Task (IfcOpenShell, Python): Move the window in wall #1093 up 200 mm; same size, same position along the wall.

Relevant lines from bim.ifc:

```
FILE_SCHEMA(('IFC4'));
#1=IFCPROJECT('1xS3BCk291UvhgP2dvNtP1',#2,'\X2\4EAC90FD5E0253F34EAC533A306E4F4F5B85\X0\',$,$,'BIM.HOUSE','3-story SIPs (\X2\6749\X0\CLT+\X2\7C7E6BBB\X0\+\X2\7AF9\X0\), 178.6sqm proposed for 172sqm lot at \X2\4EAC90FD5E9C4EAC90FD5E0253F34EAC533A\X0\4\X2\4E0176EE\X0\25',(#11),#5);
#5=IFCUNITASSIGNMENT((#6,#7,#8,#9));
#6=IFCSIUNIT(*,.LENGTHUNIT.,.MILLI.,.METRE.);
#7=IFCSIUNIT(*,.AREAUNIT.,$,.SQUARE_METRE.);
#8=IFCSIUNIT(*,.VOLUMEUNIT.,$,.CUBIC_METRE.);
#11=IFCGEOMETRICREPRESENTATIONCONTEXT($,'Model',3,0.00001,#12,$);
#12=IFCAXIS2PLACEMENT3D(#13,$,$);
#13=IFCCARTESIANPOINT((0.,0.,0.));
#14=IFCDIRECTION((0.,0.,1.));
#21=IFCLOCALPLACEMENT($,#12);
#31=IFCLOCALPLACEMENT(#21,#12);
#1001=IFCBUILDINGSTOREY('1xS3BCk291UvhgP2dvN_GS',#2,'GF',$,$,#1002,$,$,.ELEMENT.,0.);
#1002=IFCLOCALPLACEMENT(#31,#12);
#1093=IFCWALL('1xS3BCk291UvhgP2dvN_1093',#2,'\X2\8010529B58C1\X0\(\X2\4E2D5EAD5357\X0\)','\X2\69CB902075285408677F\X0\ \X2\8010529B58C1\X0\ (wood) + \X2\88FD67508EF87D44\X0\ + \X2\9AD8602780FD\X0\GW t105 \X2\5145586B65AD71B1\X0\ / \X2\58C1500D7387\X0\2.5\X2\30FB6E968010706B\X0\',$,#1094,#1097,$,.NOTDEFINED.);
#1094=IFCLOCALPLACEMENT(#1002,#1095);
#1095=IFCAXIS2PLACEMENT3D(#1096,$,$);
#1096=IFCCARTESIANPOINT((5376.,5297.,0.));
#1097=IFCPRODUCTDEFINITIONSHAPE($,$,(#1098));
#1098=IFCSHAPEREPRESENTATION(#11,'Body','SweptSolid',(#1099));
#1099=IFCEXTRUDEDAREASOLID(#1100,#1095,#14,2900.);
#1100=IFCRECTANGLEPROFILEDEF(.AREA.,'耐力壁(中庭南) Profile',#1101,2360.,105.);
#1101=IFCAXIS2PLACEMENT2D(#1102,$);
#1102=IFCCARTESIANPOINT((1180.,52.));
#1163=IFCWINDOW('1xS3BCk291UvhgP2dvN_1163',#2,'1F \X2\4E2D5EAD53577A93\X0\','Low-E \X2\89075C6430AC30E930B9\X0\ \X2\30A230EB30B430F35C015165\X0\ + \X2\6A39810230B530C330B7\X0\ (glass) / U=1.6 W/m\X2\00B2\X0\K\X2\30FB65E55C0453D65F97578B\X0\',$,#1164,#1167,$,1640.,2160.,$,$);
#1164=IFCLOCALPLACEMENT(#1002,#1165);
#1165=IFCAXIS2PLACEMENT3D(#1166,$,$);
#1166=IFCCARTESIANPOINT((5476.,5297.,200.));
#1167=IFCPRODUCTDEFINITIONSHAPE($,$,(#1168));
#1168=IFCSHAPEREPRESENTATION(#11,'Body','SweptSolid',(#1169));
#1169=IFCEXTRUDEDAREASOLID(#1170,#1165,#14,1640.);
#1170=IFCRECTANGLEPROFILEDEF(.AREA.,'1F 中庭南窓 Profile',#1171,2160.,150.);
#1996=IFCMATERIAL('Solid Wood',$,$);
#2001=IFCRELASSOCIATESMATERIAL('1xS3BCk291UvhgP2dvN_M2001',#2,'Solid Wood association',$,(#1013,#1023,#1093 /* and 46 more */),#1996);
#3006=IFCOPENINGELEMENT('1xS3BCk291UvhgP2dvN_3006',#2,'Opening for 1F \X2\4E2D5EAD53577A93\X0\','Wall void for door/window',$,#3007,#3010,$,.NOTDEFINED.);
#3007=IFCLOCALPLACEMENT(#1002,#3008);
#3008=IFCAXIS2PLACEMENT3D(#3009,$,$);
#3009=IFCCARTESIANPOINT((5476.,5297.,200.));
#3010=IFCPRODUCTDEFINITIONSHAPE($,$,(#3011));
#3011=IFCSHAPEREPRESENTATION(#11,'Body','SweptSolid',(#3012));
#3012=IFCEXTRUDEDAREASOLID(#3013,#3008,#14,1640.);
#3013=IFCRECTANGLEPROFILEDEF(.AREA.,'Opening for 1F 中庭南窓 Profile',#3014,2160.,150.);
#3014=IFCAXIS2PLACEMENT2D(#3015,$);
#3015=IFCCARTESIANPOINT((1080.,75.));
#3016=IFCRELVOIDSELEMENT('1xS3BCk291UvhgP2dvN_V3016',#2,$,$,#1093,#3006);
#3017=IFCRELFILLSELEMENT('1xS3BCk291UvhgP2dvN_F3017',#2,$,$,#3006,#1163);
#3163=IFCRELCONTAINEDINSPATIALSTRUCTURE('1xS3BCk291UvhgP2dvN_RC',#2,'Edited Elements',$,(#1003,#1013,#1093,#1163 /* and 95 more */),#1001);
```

```python
import numpy as np
import ifcopenshell
import ifcopenshell.api.geometry
import ifcopenshell.util.placement
import ifcopenshell.util.unit

model = ifcopenshell.open("bim.ifc")
unit_scale = ifcopenshell.util.unit.calculate_unit_scale(model)

window = model.by_id(1163)
opening = window.FillsVoids[0].RelatingOpeningElement
dz = 0.2 / unit_scale

shift = np.array([0.0, 0.0, dz])
# The window is not placed relative to its opening, so move both.
for product in (opening, window):
    matrix = ifcopenshell.util.placement.get_local_placement(product.ObjectPlacement)
    matrix[:3, 3] += shift
    ifcopenshell.api.geometry.edit_object_placement(model, product=product, matrix=matrix, is_si=False)

print(f"moved by {dz * unit_scale:+.3f} m")

model.write("bim-out.ifc")
```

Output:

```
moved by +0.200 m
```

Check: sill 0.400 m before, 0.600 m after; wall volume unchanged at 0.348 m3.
